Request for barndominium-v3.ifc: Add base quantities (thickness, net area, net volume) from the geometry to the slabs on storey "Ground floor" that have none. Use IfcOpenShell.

First a look at what the model holds.

```python
import ifcopenshell
import ifcopenshell.util.element
import ifcopenshell.util.unit

model = ifcopenshell.open("barndominium-v3.ifc")
print(model.schema)
for unit_type in ("LENGTHUNIT", "AREAUNIT", "VOLUMEUNIT"):
    print(unit_type, ifcopenshell.util.unit.calculate_unit_scale(model, unit_type))
storey = next(s for s in model.by_type("IfcBuildingStorey") if s.Name == "Ground floor")
slabs = [e for e in ifcopenshell.util.element.get_decomposition(storey) if e.is_a("IfcSlab")]
for e in sorted(slabs, key=lambda e: e.id()):
    print(e.id(), e.is_a(), e.Name, list(ifcopenshell.util.element.get_psets(e, qtos_only=True)), sep=" | ")
```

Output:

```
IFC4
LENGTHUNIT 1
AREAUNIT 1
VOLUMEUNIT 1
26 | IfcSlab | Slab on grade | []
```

```python
import ifcopenshell
import ifcopenshell.api.pset
import ifcopenshell.geom
import ifcopenshell.util.element
import ifcopenshell.util.shape
import ifcopenshell.util.unit

model = ifcopenshell.open("barndominium-v3.ifc")
unit_scale = ifcopenshell.util.unit.calculate_unit_scale(model)
area_scale = ifcopenshell.util.unit.calculate_unit_scale(model, "AREAUNIT")
volume_scale = ifcopenshell.util.unit.calculate_unit_scale(model, "VOLUMEUNIT")
settings = ifcopenshell.geom.settings()

storey = next(s for s in model.by_type("IfcBuildingStorey") if s.Name == "Ground floor")
slabs = [e for e in ifcopenshell.util.element.get_decomposition(storey) if e.is_a("IfcSlab")]

for e in sorted(slabs, key=lambda e: e.id()):
    if ifcopenshell.util.element.get_psets(e, qtos_only=True, should_inherit=False):
        continue
    # Geometry comes back in metres, in the element's own axes.
    shape = ifcopenshell.geom.create_shape(settings, e)
    values = {
        "Width": ifcopenshell.util.shape.get_z(shape.geometry) / unit_scale,
        "NetArea": ifcopenshell.util.shape.get_footprint_area(shape.geometry) / area_scale,
        "NetVolume": ifcopenshell.util.shape.get_volume(shape.geometry) / volume_scale,
    }
    qto = ifcopenshell.api.pset.add_qto(model, product=e, name="Qto_SlabBaseQuantities")
    ifcopenshell.api.pset.edit_qto(model, qto=qto, properties=values)
    print(e.id(), {k: round(v, 3) for k, v in values.items()})

model.write("barndominium-v3-out.ifc")
```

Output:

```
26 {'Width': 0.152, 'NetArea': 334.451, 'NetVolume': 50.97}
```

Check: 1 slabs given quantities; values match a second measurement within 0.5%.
